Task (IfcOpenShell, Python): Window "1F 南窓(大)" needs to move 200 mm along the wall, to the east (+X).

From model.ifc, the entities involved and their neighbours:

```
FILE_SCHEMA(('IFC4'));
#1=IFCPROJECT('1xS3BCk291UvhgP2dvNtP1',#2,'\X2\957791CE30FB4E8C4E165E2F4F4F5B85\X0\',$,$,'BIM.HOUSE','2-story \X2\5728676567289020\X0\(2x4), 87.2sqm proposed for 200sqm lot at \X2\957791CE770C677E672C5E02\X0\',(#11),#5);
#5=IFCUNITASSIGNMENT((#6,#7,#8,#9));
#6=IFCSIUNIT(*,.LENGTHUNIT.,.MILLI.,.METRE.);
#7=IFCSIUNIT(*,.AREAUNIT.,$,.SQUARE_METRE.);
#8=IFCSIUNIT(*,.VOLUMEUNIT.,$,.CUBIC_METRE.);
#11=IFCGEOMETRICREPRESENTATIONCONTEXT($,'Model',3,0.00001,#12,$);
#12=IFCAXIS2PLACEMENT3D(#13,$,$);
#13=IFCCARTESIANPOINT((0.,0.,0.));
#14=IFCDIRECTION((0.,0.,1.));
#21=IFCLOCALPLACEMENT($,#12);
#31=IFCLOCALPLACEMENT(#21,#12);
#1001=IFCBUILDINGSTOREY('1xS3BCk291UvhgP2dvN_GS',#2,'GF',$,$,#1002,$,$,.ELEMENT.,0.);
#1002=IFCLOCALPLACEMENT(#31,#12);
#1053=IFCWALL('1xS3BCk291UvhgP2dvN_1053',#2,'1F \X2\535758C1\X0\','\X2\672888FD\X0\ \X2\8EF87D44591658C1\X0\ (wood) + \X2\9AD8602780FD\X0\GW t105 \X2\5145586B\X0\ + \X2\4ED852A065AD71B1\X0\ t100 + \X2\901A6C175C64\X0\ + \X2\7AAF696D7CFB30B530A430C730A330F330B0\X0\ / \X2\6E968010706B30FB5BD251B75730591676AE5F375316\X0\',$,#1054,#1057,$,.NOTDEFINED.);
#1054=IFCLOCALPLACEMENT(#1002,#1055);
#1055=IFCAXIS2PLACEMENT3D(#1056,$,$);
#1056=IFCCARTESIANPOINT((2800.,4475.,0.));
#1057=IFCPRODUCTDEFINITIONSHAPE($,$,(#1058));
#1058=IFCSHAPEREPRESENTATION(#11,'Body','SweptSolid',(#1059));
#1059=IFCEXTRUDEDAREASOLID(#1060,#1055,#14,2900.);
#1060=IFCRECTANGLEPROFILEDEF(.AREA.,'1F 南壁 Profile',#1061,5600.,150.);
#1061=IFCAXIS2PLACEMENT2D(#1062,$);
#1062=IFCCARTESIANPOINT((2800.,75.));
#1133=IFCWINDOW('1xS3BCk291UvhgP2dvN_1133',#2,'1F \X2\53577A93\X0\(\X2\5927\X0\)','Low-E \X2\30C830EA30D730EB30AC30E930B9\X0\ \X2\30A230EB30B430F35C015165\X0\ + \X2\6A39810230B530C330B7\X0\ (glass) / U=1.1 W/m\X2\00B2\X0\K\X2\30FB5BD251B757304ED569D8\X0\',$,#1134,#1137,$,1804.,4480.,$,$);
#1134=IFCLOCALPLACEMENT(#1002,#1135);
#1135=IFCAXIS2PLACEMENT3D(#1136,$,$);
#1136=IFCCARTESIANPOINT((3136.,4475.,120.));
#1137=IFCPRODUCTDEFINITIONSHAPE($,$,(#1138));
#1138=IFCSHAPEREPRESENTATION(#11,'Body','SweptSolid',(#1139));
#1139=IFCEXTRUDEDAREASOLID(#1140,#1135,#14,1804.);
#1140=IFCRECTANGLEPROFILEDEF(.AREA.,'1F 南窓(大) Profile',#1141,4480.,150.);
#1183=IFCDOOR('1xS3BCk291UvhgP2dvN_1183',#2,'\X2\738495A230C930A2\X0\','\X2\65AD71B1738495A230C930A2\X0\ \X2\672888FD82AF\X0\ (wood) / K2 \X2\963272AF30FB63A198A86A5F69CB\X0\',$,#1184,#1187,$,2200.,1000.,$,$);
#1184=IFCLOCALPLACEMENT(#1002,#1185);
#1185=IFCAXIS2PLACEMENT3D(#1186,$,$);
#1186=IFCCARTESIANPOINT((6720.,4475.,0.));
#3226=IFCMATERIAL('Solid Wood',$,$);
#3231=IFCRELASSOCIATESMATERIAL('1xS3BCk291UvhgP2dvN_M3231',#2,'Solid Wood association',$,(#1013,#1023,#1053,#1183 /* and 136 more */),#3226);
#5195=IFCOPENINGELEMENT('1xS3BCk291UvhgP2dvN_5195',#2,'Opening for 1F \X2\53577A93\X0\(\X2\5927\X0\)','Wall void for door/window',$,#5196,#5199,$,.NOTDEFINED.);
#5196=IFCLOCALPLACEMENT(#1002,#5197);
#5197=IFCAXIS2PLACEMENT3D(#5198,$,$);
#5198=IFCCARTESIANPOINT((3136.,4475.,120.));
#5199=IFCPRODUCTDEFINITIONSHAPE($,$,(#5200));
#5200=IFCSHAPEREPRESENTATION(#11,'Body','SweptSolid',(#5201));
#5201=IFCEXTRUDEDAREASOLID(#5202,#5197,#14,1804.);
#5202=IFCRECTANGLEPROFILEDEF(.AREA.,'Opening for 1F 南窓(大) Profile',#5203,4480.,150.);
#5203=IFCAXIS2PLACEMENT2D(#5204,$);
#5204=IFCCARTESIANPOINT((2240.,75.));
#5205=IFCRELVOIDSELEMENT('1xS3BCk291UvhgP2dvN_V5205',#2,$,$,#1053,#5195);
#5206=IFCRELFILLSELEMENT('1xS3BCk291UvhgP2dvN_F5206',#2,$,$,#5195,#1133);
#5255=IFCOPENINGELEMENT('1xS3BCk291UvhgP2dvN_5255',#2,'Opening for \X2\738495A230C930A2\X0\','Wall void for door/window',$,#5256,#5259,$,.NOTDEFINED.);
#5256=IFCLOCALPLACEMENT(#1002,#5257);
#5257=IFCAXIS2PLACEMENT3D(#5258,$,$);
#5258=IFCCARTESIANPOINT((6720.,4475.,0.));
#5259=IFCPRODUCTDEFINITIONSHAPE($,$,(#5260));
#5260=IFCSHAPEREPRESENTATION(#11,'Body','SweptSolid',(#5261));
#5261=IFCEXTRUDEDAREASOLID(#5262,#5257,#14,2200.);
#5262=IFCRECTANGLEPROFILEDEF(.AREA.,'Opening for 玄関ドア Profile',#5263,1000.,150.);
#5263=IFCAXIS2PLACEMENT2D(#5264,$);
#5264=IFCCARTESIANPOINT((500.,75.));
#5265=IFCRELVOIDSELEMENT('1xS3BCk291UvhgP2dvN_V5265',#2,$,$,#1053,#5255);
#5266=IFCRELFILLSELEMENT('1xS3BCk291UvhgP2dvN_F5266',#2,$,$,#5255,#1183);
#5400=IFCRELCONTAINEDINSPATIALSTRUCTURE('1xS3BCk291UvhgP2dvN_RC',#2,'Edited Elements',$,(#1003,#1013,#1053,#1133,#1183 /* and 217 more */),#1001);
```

```python
import ifcopenshell
import ifcopenshell.api.geometry
import ifcopenshell.util.placement
import ifcopenshell.util.unit

model = ifcopenshell.open("model.ifc")
unit_scale = ifcopenshell.util.unit.calculate_unit_scale(model)

window = model.by_guid("1xS3BCk291UvhgP2dvN_1133")
opening = window.FillsVoids[0].RelatingOpeningElement
wall = opening.VoidsElements[0].RelatingBuildingElement

wall_matrix = ifcopenshell.util.placement.get_local_placement(wall.ObjectPlacement)
shift = wall_matrix[:3, 0] * 0.2 / unit_scale
before = ifcopenshell.util.placement.get_local_placement(window.ObjectPlacement)[:3, 3].copy()

# The window is not placed relative to its opening, so move both.
for product in (opening, window):
    matrix = ifcopenshell.util.placement.get_local_placement(product.ObjectPlacement)
    matrix[:3, 3] += shift
    ifcopenshell.api.geometry.edit_object_placement(model, product=product, matrix=matrix, is_si=False)

after = ifcopenshell.util.placement.get_local_placement(window.ObjectPlacement)[:3, 3]
print("window moved by", (after - before).round(3) + 0.0)

model.write("model_v2.ifc")
```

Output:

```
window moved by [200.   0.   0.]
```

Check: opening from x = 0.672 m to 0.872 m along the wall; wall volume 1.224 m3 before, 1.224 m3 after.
